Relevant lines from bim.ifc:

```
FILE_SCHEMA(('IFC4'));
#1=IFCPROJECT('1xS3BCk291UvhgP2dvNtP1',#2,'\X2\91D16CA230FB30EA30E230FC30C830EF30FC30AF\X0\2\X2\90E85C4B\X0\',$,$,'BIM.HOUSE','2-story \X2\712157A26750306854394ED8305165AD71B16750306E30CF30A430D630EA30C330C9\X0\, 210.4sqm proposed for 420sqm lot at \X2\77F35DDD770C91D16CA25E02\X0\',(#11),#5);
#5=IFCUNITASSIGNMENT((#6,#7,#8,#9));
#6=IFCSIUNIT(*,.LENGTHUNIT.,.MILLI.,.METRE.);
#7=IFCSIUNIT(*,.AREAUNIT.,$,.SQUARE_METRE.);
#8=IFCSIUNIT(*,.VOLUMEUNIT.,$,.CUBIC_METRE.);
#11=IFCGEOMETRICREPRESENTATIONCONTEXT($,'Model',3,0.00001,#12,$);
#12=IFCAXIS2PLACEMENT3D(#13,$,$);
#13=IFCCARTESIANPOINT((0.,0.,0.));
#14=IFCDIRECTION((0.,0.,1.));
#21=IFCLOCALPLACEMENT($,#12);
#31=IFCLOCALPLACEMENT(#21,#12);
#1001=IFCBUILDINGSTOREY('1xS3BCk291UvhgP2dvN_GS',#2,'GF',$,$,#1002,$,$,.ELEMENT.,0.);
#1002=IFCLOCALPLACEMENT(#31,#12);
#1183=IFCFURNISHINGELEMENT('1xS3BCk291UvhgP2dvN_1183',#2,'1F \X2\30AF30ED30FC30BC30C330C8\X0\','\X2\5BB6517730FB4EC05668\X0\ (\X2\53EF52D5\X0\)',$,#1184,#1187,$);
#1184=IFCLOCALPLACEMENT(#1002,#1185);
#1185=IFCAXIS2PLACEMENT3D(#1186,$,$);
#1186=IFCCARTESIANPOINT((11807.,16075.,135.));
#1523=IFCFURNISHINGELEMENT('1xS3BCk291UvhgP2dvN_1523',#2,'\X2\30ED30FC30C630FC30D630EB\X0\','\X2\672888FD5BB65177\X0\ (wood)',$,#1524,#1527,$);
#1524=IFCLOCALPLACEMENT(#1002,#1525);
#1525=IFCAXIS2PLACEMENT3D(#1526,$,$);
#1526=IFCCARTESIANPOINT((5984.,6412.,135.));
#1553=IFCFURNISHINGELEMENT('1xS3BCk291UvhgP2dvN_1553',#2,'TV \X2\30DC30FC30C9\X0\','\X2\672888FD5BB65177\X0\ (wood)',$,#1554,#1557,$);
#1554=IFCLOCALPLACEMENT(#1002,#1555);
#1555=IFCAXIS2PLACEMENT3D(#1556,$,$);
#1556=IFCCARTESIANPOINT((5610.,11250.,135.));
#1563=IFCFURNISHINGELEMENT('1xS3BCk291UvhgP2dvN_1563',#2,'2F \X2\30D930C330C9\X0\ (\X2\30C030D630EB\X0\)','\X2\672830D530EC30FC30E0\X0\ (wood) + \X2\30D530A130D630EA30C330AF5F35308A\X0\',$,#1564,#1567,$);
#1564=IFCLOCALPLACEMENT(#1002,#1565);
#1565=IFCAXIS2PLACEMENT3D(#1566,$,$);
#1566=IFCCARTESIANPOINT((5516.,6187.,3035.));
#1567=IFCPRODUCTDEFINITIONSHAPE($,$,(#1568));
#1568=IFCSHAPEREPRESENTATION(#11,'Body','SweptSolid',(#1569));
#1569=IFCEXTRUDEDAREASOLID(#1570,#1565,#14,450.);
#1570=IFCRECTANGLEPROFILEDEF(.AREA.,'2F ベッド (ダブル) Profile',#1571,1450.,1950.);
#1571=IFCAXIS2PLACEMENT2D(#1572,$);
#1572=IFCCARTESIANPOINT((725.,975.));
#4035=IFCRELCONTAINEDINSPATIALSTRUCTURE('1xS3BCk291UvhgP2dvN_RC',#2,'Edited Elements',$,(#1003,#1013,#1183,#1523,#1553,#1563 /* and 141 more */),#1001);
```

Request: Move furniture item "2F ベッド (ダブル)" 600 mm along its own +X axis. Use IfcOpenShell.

```python
import ifcopenshell
import ifcopenshell.api.geometry
import ifcopenshell.util.placement
import ifcopenshell.util.unit

model = ifcopenshell.open("bim.ifc")
unit_scale = ifcopenshell.util.unit.calculate_unit_scale(model)

item = model.by_guid("1xS3BCk291UvhgP2dvN_1563")
matrix = ifcopenshell.util.placement.get_local_placement(item.ObjectPlacement)
matrix[:3, 3] += matrix[:3, 0] * 0.6 / unit_scale
ifcopenshell.api.geometry.edit_object_placement(model, product=item, matrix=matrix, is_si=False)

print(ifcopenshell.util.placement.get_local_placement(item.ObjectPlacement).round(3) + 0.0)

model.write("bim_v2.ifc")
```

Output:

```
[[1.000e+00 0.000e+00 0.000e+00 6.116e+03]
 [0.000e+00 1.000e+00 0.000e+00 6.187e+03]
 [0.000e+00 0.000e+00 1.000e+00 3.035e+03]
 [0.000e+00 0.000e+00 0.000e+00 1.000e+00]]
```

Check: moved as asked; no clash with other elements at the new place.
